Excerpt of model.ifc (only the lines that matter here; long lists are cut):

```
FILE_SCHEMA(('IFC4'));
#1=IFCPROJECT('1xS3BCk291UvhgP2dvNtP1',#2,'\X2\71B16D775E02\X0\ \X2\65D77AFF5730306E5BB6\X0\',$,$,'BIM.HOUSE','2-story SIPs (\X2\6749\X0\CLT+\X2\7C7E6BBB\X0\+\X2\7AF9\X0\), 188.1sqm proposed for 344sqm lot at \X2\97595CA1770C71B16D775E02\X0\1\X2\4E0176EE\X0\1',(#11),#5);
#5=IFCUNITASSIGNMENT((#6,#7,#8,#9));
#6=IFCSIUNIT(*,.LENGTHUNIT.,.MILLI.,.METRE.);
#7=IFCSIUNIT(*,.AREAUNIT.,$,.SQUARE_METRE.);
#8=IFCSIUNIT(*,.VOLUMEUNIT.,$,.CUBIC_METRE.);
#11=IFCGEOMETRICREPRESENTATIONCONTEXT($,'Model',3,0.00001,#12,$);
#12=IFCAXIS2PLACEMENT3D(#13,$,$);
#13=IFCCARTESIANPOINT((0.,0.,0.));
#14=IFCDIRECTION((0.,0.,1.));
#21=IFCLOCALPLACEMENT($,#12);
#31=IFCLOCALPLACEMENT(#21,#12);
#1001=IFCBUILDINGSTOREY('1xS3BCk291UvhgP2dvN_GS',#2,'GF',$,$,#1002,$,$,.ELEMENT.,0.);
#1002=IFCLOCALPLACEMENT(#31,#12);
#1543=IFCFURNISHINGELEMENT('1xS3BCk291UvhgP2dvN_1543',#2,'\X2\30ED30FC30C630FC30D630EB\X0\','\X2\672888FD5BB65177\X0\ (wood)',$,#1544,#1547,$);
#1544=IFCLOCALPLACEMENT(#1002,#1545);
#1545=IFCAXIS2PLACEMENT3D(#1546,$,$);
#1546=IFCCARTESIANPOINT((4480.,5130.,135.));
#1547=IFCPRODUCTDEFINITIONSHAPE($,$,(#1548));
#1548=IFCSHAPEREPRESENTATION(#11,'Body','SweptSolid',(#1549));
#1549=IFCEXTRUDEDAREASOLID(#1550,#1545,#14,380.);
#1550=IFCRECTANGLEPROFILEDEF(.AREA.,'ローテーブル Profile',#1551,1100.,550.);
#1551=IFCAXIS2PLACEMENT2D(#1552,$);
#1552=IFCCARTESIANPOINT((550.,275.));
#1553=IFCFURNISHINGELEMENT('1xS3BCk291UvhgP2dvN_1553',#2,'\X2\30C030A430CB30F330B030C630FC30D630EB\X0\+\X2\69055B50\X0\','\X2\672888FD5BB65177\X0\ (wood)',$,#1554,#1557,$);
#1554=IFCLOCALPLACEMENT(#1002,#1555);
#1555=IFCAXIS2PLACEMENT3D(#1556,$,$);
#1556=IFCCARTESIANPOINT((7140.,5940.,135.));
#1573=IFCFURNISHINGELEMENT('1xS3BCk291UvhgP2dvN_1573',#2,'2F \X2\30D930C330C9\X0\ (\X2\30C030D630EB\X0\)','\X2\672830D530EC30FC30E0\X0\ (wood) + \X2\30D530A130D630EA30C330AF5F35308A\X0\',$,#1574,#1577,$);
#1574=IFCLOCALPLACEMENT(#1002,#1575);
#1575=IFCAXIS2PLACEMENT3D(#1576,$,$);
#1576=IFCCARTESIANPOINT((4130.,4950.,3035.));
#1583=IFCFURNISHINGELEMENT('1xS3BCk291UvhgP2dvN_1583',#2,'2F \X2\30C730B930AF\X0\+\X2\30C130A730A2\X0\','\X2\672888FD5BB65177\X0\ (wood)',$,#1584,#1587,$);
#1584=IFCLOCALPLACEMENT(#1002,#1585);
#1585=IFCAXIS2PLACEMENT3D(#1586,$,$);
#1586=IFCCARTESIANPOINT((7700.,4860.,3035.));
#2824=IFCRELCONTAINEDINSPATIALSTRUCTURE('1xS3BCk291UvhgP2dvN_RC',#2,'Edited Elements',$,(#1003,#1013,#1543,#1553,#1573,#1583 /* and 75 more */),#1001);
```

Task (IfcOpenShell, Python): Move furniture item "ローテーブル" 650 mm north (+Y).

```python
import ifcopenshell
import ifcopenshell.api.geometry
import ifcopenshell.util.placement
import ifcopenshell.util.unit

model = ifcopenshell.open("model.ifc")
unit_scale = ifcopenshell.util.unit.calculate_unit_scale(model)

item = model.by_guid("1xS3BCk291UvhgP2dvN_1543")
matrix = ifcopenshell.util.placement.get_local_placement(item.ObjectPlacement)
matrix[1, 3] += 0.65 / unit_scale
ifcopenshell.api.geometry.edit_object_placement(model, product=item, matrix=matrix, is_si=False)

print(ifcopenshell.util.placement.get_local_placement(item.ObjectPlacement).round(3) + 0.0)

model.write("model-out.ifc")
```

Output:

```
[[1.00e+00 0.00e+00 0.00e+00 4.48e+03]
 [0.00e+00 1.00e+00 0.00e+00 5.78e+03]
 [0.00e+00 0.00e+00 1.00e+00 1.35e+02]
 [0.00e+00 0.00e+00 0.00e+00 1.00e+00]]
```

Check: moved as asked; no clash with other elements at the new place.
